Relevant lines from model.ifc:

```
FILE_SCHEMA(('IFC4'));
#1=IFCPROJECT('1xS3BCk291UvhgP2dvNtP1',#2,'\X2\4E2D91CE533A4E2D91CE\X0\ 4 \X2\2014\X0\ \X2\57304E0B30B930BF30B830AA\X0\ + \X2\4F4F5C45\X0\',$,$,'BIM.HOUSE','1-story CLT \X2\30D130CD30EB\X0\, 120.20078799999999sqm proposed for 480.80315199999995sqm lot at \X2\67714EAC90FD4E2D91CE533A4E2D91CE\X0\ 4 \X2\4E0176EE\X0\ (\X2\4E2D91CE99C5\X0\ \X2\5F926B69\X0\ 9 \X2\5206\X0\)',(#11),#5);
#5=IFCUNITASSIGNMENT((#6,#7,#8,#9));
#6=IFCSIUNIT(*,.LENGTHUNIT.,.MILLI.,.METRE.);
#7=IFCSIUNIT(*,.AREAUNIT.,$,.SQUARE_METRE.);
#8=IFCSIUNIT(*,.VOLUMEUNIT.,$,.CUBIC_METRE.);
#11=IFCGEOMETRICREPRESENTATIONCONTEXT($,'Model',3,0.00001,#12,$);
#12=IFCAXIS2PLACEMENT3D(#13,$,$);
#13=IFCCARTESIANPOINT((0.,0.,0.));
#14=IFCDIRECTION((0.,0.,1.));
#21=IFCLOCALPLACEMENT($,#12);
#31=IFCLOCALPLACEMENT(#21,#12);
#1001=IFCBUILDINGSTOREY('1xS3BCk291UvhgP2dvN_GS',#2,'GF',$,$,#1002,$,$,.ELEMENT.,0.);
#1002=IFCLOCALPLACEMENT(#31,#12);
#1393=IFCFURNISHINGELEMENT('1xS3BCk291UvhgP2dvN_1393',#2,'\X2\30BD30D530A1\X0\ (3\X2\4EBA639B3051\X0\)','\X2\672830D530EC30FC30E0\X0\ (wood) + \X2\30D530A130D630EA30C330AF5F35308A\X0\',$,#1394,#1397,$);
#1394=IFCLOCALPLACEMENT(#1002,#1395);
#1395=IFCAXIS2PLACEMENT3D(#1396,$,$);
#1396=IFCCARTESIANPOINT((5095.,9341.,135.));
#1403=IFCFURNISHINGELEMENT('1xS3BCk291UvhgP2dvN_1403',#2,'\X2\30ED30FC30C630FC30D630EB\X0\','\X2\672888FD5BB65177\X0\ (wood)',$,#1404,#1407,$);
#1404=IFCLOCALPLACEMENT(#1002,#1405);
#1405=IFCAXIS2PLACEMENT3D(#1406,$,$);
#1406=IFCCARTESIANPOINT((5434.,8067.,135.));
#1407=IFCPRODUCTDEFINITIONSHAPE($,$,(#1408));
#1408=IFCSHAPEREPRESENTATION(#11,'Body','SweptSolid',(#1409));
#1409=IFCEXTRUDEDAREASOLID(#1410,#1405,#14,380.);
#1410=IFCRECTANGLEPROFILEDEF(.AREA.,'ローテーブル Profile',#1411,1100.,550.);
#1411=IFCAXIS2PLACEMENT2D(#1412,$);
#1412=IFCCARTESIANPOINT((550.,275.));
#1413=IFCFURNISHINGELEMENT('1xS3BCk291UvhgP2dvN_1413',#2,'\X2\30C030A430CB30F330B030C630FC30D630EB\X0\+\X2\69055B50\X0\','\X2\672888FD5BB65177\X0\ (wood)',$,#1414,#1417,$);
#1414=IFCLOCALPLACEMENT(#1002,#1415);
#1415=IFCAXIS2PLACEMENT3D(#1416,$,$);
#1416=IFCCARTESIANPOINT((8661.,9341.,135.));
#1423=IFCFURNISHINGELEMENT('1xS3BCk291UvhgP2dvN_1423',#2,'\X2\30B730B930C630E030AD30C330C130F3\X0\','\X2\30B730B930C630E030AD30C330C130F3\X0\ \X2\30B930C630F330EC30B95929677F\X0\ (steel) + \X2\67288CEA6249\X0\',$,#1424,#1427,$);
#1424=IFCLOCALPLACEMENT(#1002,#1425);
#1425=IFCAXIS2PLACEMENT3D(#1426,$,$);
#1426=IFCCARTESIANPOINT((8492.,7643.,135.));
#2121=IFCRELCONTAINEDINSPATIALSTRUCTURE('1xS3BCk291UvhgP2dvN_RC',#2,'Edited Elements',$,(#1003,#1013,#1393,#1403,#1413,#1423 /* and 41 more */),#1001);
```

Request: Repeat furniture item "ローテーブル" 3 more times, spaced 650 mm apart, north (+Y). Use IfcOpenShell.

```python
import numpy as np
import ifcopenshell
import ifcopenshell.api.geometry
import ifcopenshell.api.root
import ifcopenshell.util.element
import ifcopenshell.util.placement

model = ifcopenshell.open("model.ifc")


def reuse_history(source, copy):
    """copy_class also copies each property set's owner history, people and application; keep the originals."""
    for rel in copy.IsDefinedBy:
        if rel.is_a("IfcRelDefinesByProperties") and (history := rel.RelatingPropertyDefinition.OwnerHistory):
            rel.RelatingPropertyDefinition.OwnerHistory = source.OwnerHistory
            ifcopenshell.util.element.remove_deep2(model, history)


source = model.by_guid("1xS3BCk291UvhgP2dvN_1403")
base = ifcopenshell.util.placement.get_local_placement(source.ObjectPlacement)
step = np.array([0.0, 1.0, 0.0]) * 650.0

for i in range(1, 4):
    copy = ifcopenshell.api.root.copy_class(model, product=source)
    copy.Representation = ifcopenshell.util.element.copy_deep(
        model, source.Representation, exclude=["IfcGeometricRepresentationContext", "IfcRepresentationMap"]
    )
    reuse_history(source, copy)
    matrix = base.copy()
    matrix[:3, 3] += i * step
    print("added at", matrix[:3, 3].round(3) + 0.0)
    ifcopenshell.api.geometry.edit_object_placement(model, product=copy, matrix=matrix, is_si=False)

model.write("model_v2.ifc")
```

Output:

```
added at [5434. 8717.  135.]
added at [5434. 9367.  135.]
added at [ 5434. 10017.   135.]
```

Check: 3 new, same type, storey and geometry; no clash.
